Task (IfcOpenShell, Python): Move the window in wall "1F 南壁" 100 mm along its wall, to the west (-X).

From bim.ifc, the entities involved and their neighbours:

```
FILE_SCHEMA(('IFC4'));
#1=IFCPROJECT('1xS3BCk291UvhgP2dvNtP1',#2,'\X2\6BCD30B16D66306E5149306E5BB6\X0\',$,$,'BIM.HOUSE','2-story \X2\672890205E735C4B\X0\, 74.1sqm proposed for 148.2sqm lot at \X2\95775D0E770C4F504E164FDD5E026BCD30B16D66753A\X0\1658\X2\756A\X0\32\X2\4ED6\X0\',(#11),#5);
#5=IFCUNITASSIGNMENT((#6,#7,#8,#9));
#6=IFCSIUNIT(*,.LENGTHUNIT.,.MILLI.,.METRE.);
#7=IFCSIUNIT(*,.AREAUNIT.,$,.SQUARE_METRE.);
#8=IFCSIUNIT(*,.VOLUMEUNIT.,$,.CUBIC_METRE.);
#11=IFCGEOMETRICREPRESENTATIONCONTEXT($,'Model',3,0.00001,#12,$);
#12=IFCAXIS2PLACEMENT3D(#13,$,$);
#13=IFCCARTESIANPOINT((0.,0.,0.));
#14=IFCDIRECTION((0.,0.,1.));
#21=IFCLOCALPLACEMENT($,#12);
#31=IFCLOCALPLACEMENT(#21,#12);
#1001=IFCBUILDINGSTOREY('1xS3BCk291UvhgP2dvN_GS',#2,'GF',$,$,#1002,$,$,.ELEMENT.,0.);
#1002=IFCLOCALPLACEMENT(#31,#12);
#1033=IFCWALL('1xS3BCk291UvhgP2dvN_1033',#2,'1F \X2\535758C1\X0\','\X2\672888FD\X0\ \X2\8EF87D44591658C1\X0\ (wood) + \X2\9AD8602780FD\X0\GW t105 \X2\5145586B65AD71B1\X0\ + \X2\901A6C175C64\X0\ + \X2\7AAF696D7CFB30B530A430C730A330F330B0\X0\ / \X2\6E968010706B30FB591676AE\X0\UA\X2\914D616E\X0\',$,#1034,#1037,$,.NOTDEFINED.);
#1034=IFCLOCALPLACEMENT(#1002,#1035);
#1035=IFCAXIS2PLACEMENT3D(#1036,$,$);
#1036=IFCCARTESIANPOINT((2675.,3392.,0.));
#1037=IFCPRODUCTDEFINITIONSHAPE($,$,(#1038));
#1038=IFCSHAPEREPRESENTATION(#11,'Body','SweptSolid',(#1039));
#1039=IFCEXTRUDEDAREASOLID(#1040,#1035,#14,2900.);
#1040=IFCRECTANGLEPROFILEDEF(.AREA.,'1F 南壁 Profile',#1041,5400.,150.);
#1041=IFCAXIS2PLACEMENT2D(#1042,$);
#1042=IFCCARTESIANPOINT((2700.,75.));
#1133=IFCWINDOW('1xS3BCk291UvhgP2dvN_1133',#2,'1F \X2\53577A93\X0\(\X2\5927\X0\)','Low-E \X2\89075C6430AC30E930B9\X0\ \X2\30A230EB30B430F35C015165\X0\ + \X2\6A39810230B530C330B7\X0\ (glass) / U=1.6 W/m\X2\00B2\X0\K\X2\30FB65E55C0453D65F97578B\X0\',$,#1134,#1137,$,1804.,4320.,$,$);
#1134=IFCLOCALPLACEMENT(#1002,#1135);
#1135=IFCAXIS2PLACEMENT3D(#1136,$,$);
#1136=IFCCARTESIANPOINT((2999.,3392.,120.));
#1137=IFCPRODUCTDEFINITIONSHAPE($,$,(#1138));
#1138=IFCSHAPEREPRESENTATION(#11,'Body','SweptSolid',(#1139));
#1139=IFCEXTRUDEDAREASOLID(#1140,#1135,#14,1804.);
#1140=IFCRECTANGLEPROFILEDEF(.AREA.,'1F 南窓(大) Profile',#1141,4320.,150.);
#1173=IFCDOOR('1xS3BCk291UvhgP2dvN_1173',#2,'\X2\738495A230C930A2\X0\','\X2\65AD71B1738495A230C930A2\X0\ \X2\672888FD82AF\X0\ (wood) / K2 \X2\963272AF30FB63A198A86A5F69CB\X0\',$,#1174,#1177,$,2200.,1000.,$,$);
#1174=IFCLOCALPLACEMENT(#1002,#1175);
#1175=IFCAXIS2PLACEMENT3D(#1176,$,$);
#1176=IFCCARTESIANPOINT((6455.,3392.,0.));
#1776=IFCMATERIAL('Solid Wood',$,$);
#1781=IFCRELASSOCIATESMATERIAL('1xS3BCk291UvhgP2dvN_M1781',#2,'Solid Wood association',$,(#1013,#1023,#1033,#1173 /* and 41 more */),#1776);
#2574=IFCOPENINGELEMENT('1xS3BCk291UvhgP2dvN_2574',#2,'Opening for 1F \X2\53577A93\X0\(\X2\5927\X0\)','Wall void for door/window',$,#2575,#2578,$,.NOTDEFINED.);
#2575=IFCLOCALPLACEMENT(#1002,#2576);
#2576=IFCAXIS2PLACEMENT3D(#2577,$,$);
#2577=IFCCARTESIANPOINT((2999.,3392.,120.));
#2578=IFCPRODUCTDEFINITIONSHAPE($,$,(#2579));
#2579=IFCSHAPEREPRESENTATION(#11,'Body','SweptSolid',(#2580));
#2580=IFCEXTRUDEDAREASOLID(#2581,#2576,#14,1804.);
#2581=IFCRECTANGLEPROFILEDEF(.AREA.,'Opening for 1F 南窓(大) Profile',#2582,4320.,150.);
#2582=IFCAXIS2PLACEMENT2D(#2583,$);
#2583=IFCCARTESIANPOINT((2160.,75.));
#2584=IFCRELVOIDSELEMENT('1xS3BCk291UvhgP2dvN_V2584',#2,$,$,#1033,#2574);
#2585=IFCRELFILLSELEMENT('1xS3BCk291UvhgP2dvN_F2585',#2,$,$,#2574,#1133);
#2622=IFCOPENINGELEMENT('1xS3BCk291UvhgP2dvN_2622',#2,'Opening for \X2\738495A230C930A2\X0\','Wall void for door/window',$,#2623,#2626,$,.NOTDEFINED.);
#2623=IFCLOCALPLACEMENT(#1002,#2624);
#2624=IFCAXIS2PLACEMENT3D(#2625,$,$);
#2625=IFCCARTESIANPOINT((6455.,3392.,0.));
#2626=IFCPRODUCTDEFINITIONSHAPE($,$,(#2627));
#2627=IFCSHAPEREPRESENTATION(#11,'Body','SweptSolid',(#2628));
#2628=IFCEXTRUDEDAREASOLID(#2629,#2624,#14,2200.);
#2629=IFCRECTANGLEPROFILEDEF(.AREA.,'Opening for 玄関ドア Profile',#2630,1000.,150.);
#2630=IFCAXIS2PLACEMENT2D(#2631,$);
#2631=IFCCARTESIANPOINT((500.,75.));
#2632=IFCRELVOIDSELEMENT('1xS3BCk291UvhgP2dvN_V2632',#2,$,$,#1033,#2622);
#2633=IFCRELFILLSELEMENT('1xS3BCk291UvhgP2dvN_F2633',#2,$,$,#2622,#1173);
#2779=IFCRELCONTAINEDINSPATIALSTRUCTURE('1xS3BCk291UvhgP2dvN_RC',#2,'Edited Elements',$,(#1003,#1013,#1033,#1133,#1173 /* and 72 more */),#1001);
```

```python
import ifcopenshell
import ifcopenshell.api.geometry
import ifcopenshell.util.placement
import ifcopenshell.util.unit

model = ifcopenshell.open("bim.ifc")
unit_scale = ifcopenshell.util.unit.calculate_unit_scale(model)

window = model.by_guid("1xS3BCk291UvhgP2dvN_1133")
opening = window.FillsVoids[0].RelatingOpeningElement
wall = opening.VoidsElements[0].RelatingBuildingElement

wall_matrix = ifcopenshell.util.placement.get_local_placement(wall.ObjectPlacement)
shift = wall_matrix[:3, 0] * -0.1 / unit_scale
before = ifcopenshell.util.placement.get_local_placement(window.ObjectPlacement)[:3, 3].copy()

# The window is not placed relative to its opening, so move both.
for product in (opening, window):
    matrix = ifcopenshell.util.placement.get_local_placement(product.ObjectPlacement)
    matrix[:3, 3] += shift
    ifcopenshell.api.geometry.edit_object_placement(model, product=product, matrix=matrix, is_si=False)

after = ifcopenshell.util.placement.get_local_placement(window.ObjectPlacement)[:3, 3]
print("window moved by", (after - before).round(3) + 0.0)

model.write("bim_rev.ifc")
```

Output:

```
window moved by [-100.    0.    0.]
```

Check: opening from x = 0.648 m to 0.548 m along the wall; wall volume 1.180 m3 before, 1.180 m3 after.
